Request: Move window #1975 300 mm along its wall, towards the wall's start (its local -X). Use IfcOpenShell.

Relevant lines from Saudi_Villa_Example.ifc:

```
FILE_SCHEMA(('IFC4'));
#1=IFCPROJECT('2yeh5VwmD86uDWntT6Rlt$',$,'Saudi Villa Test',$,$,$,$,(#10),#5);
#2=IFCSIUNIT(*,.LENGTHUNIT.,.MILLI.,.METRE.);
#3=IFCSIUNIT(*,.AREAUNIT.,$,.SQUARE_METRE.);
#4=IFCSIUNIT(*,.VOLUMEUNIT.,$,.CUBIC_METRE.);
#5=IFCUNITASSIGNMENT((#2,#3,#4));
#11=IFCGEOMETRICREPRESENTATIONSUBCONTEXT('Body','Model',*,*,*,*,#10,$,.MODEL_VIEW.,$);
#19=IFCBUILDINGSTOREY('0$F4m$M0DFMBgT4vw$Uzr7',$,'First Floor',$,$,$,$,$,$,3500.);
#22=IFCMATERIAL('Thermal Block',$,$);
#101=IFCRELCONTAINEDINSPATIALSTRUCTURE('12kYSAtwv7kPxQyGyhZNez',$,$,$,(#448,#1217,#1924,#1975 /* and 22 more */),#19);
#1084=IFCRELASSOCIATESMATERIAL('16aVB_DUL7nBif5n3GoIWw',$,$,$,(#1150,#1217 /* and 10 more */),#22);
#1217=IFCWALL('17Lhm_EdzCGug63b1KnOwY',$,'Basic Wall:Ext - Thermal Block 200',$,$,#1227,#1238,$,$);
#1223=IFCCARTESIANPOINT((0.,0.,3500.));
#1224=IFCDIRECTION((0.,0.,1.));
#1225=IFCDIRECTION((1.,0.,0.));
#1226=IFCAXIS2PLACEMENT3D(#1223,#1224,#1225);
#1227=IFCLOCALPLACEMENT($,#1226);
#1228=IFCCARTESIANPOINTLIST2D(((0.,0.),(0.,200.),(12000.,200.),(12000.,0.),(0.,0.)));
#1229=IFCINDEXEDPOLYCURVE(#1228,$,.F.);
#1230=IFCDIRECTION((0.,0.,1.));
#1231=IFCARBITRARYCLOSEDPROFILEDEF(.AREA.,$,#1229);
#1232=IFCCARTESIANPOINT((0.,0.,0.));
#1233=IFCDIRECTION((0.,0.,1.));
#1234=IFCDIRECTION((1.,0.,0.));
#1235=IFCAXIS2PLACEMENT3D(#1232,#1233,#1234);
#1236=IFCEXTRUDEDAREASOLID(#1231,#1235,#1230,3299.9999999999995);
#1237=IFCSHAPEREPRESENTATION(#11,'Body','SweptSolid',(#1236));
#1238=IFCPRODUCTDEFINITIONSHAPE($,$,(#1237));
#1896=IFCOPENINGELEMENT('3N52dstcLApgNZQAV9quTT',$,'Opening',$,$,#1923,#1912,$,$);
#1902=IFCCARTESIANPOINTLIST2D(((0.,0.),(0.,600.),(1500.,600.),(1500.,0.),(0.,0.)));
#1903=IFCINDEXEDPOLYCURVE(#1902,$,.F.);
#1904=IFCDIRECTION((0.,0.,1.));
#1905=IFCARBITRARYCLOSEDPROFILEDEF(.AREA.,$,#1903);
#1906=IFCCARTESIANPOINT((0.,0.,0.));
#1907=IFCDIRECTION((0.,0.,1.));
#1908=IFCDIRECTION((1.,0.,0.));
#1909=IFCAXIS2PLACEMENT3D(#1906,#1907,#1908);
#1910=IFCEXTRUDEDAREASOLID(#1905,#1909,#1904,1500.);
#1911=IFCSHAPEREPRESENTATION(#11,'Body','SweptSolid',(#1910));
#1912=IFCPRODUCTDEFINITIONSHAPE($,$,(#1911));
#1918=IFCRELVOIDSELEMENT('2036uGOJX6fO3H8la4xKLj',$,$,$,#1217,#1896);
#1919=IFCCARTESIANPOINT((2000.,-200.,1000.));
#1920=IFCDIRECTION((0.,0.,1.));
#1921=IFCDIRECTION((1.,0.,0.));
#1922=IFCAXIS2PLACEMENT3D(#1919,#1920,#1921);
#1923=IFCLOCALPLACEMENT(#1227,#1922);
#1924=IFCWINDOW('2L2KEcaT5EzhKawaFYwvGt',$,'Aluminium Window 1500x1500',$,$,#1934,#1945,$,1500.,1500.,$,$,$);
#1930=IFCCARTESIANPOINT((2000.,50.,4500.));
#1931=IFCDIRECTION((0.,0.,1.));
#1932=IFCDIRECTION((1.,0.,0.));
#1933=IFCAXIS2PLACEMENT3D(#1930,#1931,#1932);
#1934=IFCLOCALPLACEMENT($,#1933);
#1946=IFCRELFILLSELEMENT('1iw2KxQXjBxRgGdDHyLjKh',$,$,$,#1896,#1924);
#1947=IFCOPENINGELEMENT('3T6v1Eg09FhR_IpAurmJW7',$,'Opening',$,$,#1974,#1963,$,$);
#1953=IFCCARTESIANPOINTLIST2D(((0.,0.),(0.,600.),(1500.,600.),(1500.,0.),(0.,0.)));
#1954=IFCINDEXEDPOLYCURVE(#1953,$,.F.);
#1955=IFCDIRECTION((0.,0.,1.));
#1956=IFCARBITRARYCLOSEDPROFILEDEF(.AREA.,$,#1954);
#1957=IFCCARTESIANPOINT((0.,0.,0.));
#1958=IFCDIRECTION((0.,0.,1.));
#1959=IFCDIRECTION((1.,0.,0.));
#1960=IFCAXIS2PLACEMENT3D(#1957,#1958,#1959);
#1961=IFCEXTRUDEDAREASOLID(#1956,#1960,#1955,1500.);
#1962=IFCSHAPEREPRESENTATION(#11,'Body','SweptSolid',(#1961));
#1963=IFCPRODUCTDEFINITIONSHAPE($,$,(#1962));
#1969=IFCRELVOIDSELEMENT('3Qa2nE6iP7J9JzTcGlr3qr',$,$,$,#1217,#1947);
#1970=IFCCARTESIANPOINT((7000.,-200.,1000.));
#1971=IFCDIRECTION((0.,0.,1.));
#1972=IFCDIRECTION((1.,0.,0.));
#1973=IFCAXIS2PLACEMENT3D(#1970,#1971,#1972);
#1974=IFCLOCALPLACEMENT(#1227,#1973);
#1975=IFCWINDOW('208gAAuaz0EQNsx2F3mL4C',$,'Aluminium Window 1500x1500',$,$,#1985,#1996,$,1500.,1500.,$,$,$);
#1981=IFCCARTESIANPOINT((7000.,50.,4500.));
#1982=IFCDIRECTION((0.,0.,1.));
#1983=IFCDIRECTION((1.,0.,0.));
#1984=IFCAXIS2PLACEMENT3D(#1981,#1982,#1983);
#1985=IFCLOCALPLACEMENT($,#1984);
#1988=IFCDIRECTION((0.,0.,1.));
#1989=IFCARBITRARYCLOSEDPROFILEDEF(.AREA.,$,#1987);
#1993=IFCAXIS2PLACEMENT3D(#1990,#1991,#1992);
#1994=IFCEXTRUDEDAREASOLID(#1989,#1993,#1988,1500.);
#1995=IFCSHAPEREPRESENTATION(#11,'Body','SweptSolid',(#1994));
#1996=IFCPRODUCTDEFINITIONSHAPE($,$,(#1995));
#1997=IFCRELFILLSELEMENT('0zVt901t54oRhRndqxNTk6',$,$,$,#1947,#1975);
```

```python
import ifcopenshell
import ifcopenshell.api.geometry
import ifcopenshell.util.placement
import ifcopenshell.util.unit

model = ifcopenshell.open("Saudi_Villa_Example.ifc")
unit_scale = ifcopenshell.util.unit.calculate_unit_scale(model)

window = model.by_guid("208gAAuaz0EQNsx2F3mL4C")
opening = window.FillsVoids[0].RelatingOpeningElement
wall = opening.VoidsElements[0].RelatingBuildingElement

wall_matrix = ifcopenshell.util.placement.get_local_placement(wall.ObjectPlacement)
shift = wall_matrix[:3, 0] * -0.3 / unit_scale
before = ifcopenshell.util.placement.get_local_placement(window.ObjectPlacement)[:3, 3].copy()

# The window is not placed relative to its opening, so move both.
for product in (opening, window):
    matrix = ifcopenshell.util.placement.get_local_placement(product.ObjectPlacement)
    matrix[:3, 3] += shift
    ifcopenshell.api.geometry.edit_object_placement(model, product=product, matrix=matrix, is_si=False)

after = ifcopenshell.util.placement.get_local_placement(window.ObjectPlacement)[:3, 3]
print("window moved by", (after - before).round(3) + 0.0)

model.write("Saudi_Villa_Example_edited.ifc")
```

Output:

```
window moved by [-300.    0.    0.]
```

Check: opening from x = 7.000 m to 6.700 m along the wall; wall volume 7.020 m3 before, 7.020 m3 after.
